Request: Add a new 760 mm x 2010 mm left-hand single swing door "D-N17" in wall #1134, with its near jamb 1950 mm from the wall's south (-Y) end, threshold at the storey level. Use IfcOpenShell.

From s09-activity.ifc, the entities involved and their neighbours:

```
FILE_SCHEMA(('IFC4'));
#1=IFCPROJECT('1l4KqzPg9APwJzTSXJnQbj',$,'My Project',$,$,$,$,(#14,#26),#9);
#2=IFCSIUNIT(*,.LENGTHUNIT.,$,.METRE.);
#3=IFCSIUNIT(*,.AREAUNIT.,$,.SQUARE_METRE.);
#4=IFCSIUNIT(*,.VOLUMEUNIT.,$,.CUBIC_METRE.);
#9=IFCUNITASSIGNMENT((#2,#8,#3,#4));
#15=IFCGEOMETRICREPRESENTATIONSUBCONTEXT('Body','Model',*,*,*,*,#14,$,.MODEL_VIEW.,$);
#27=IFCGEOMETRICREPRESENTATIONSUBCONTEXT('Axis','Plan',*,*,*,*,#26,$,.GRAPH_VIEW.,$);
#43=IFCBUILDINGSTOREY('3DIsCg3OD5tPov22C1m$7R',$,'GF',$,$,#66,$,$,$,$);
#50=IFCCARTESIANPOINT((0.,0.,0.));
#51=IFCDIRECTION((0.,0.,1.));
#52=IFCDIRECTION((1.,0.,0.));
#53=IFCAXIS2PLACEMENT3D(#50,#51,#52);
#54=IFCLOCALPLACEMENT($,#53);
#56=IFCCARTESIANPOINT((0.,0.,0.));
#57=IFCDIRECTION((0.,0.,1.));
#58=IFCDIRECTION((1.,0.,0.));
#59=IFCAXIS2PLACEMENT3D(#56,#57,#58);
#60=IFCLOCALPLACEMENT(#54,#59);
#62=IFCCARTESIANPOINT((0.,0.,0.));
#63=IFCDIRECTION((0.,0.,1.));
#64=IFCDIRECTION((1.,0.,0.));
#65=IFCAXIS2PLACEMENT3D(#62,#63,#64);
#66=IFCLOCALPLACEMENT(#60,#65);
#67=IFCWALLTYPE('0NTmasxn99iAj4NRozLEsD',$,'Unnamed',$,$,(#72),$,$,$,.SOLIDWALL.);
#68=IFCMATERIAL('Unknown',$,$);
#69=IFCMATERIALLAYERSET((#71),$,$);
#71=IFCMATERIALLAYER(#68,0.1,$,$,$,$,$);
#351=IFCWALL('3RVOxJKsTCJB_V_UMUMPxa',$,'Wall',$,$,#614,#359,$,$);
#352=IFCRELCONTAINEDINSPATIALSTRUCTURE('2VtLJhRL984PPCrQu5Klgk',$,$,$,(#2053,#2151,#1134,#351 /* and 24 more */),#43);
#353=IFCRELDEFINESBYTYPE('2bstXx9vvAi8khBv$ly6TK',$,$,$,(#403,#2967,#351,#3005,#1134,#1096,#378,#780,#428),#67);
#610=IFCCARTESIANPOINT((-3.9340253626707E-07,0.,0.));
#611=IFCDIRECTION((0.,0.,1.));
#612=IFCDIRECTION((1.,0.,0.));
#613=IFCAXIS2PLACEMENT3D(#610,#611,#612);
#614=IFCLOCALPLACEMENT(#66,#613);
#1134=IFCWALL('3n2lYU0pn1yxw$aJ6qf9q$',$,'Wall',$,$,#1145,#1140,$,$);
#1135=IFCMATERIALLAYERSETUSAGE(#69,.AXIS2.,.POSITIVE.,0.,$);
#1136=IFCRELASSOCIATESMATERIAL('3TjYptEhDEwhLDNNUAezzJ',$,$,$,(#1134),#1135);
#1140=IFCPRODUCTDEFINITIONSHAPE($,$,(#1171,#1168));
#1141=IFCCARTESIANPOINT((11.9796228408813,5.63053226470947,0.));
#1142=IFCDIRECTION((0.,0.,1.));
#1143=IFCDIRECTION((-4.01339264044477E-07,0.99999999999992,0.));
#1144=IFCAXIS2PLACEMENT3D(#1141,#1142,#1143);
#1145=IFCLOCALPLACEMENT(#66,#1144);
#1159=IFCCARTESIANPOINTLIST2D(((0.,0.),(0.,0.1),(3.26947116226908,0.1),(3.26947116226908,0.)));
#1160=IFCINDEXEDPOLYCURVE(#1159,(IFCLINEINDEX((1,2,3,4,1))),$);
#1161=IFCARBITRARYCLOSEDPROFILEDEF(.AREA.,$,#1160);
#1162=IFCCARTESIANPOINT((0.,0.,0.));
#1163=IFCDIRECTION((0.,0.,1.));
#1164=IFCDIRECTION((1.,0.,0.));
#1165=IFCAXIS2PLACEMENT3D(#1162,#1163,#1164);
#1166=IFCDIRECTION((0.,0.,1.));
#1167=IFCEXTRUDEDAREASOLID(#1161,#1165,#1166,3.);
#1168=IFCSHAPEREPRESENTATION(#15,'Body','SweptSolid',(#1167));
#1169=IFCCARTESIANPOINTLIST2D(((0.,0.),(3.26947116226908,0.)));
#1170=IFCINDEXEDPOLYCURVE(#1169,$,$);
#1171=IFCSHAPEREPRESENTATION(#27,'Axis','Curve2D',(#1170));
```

```python
import numpy as np
import ifcopenshell
import ifcopenshell.api.feature
import ifcopenshell.api.geometry
import ifcopenshell.api.root
import ifcopenshell.api.spatial
import ifcopenshell.geom
import ifcopenshell.util.element
import ifcopenshell.util.placement
import ifcopenshell.util.representation
import ifcopenshell.util.shape
import ifcopenshell.util.unit

model = ifcopenshell.open("s09-activity.ifc")
unit_scale = ifcopenshell.util.unit.calculate_unit_scale(model)
settings = ifcopenshell.geom.settings()


def volume(element):
    """Net volume in cubic metres, openings subtracted."""
    shape = ifcopenshell.geom.create_shape(settings, element)
    return ifcopenshell.util.shape.get_volume(shape.geometry)


wall = model.by_id(1134)
storey = ifcopenshell.util.element.get_container(wall, ifc_class="IfcBuildingStorey")
context = ifcopenshell.util.representation.get_context(model, "Model", "Body", "MODEL_VIEW")
before = volume(wall)

width, height, from_end, sill = 0.76, 2.01, 1.95, 0.0  # metres

# The wall runs along its own X axis, and the end named is its -X end.
wall_shape = ifcopenshell.geom.create_shape(settings, wall)
x, y, z = ifcopenshell.util.shape.get_vertices(wall_shape.geometry).T
start = x.min() + from_end
face, thickness = float(y.min()), float(y.max() - y.min())
wall_matrix = ifcopenshell.util.placement.get_local_placement(wall.ObjectPlacement)
level = ifcopenshell.util.placement.get_local_placement(storey.ObjectPlacement)[2, 3]


def in_wall(x, y):
    """Placement at x, y metres in the wall's axes, at sill height."""
    matrix = wall_matrix.copy()
    matrix[:, 3] = wall_matrix @ np.array([x / unit_scale, y / unit_scale, 0.0, 1.0])
    matrix[2, 3] = level + sill / unit_scale
    return matrix


# Opening: a box that overshoots both wall faces by 50 mm.
opening = ifcopenshell.api.root.create_entity(model, ifc_class="IfcOpeningElement", predefined_type="OPENING")
box = ifcopenshell.api.geometry.add_wall_representation(
    model, context=context, length=width, height=height, thickness=thickness + 0.1
)
ifcopenshell.api.geometry.assign_representation(model, product=opening, representation=box)
ifcopenshell.api.geometry.edit_object_placement(model, product=opening, matrix=in_wall(start, face - 0.05), is_si=False)
ifcopenshell.api.feature.add_feature(model, feature=opening, element=wall)

door = ifcopenshell.api.root.create_entity(model, ifc_class="IfcDoor", name="D-N17", predefined_type="DOOR")
door.OverallWidth, door.OverallHeight = width / unit_scale, height / unit_scale
door.OperationType = "SINGLE_SWING_LEFT"
body = ifcopenshell.api.geometry.add_door_representation(
    model,
    context=context,
    overall_width=door.OverallWidth,
    overall_height=door.OverallHeight,
    operation_type="SINGLE_SWING_LEFT",
    lining_properties={"LiningDepth": thickness / unit_scale, "ThresholdDepth": thickness / unit_scale},
)
ifcopenshell.api.geometry.assign_representation(model, product=door, representation=body)
ifcopenshell.api.spatial.assign_container(model, products=[door], relating_structure=storey)
ifcopenshell.api.feature.add_filling(model, opening=opening, element=door)

# The lining spans the wall, so the door starts at the wall face.
ifcopenshell.api.geometry.edit_object_placement(model, product=door, matrix=in_wall(start, face), is_si=False)

after = volume(wall)

print(f"wall volume {before:.3f} -> {after:.3f} m3")

model.write("s09-activity_rev.ifc")
```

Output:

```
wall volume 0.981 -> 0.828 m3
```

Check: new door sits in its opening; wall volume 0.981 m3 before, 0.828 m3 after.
